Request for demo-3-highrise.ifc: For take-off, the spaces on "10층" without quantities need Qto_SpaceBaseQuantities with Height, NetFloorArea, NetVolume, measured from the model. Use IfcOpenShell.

First a look at what the model holds.

```python
import ifcopenshell
import ifcopenshell.util.element
import ifcopenshell.util.unit

model = ifcopenshell.open("demo-3-highrise.ifc")
print(model.schema)
for unit_type in ("LENGTHUNIT", "AREAUNIT", "VOLUMEUNIT"):
    print(unit_type, ifcopenshell.util.unit.calculate_unit_scale(model, unit_type))
storey = next(s for s in model.by_type("IfcBuildingStorey") if s.Name == "10층")
spaces = [e for e in ifcopenshell.util.element.get_decomposition(storey) if e.is_a("IfcSpace")]
for e in sorted(spaces, key=lambda e: e.id()):
    print(e.id(), e.is_a(), e.Name, list(ifcopenshell.util.element.get_psets(e, qtos_only=True)), sep=" | ")
```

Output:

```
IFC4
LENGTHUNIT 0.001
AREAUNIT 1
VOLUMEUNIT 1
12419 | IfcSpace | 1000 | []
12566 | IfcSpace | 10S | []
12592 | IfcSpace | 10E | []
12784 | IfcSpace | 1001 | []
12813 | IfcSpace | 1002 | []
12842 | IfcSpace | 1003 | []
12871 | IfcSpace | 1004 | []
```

```python
import ifcopenshell
import ifcopenshell.api.pset
import ifcopenshell.geom
import ifcopenshell.util.element
import ifcopenshell.util.shape
import ifcopenshell.util.unit

model = ifcopenshell.open("demo-3-highrise.ifc")
unit_scale = ifcopenshell.util.unit.calculate_unit_scale(model)
area_scale = ifcopenshell.util.unit.calculate_unit_scale(model, "AREAUNIT")
volume_scale = ifcopenshell.util.unit.calculate_unit_scale(model, "VOLUMEUNIT")
settings = ifcopenshell.geom.settings()

storey = next(s for s in model.by_type("IfcBuildingStorey") if s.Name == "10층")
spaces = [e for e in ifcopenshell.util.element.get_decomposition(storey) if e.is_a("IfcSpace")]

for e in sorted(spaces, key=lambda e: e.id()):
    if ifcopenshell.util.element.get_psets(e, qtos_only=True, should_inherit=False):
        continue
    # Geometry comes back in metres, in the element's own axes.
    shape = ifcopenshell.geom.create_shape(settings, e)
    values = {
        "Height": ifcopenshell.util.shape.get_z(shape.geometry) / unit_scale,
        "NetFloorArea": ifcopenshell.util.shape.get_footprint_area(shape.geometry) / area_scale,
        "NetVolume": ifcopenshell.util.shape.get_volume(shape.geometry) / volume_scale,
    }
    qto = ifcopenshell.api.pset.add_qto(model, product=e, name="Qto_SpaceBaseQuantities")
    ifcopenshell.api.pset.edit_qto(model, qto=qto, properties=values)
    print(e.id(), {k: round(v, 3) for k, v in values.items()})

model.write("demo-3-highrise_v2.ifc")
```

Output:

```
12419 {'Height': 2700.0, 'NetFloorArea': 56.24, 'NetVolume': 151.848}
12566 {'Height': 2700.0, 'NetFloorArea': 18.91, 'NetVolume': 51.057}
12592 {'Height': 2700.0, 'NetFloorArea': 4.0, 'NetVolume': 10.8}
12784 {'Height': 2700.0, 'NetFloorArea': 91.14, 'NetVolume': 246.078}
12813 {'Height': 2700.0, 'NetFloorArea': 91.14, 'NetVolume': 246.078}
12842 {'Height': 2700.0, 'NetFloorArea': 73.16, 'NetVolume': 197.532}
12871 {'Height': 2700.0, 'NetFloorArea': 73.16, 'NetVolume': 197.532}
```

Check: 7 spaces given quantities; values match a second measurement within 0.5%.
